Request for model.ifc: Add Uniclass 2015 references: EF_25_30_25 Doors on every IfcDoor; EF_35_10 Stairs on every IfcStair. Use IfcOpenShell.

First a look at what the model holds.

```python
import ifcopenshell

model = ifcopenshell.open("model.ifc")
print(model.schema)
print("classifications:", [c.Name for c in model.by_type("IfcClassification")])
for ifc_class in ("IfcDoor", "IfcRoof", "IfcStair", "IfcWall", "IfcWindow"):
    print(ifc_class, len(model.by_type(ifc_class)))
```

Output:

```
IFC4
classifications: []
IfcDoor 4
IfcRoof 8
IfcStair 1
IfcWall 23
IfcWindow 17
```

```python
import ifcopenshell
import ifcopenshell.api.classification

model = ifcopenshell.open("model.ifc")

system = ifcopenshell.api.classification.add_classification(model, classification="Uniclass 2015")

codes = {
    "IfcDoor": ("EF_25_30_25", "Doors"),
    "IfcStair": ("EF_35_10", "Stairs"),
}
for ifc_class, (code, name) in codes.items():
    products = model.by_type(ifc_class)
    ifcopenshell.api.classification.add_reference(
        model, products=products, classification=system, identification=code, name=name
    )
    print(code, len(products))

model.write("model_v2.ifc")
```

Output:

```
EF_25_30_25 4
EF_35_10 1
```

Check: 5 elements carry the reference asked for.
